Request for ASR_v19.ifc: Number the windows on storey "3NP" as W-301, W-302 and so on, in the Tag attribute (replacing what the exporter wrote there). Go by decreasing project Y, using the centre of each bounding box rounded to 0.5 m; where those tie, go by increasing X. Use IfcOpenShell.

First a look at what the model holds.

```python
import ifcopenshell
import ifcopenshell.util.element
import ifcopenshell.util.placement

model = ifcopenshell.open("ASR_v19.ifc")
print(model.schema)
storey = next(s for s in model.by_type("IfcBuildingStorey") if s.Name == "3NP")
windows = [e for e in ifcopenshell.util.element.get_decomposition(storey) if e.is_a("IfcWindow")]
for e in sorted(windows, key=lambda e: e.id()):
    origin = ifcopenshell.util.placement.get_local_placement(e.ObjectPlacement)[:3, 3]
    print(e.id(), e.Tag, e.Name, origin.round(2) + 0.0, sep=" | ")
```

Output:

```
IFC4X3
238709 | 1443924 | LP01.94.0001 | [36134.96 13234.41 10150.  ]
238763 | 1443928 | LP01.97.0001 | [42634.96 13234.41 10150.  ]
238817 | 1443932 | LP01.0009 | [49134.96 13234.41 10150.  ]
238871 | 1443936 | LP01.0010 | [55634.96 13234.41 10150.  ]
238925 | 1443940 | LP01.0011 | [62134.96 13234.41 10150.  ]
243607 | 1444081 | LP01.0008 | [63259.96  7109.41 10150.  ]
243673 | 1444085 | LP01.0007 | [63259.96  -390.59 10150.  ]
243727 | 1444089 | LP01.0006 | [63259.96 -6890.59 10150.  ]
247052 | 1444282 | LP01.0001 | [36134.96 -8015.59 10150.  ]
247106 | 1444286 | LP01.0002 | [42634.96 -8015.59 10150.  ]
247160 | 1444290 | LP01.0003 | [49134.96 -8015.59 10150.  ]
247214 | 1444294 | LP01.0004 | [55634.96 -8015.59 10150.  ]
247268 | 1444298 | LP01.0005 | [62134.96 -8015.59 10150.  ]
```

```python
import ifcopenshell
import ifcopenshell.geom
import ifcopenshell.util.element
import ifcopenshell.util.shape

model = ifcopenshell.open("ASR_v19.ifc")
settings = ifcopenshell.geom.settings()
settings.set("use-world-coords", True)


def centre(element):
    shape = ifcopenshell.geom.create_shape(settings, element)
    return ifcopenshell.util.shape.get_bbox_centroid(shape.geometry)


storey = next(s for s in model.by_type("IfcBuildingStorey") if s.Name == "3NP")
windows = [e for e in ifcopenshell.util.element.get_decomposition(storey) if e.is_a("IfcWindow")]

# Insertion points can sit at a corner or the storey origin, so sort by the geometry (in metres).
centres = {e: centre(e) for e in windows}
windows.sort(key=lambda e: (-round(centres[e][1] / 0.5), centres[e][0]))

for i, e in enumerate(windows, start=1):
    number = f"W-3{i:02d}"
    e.Tag = number
    print(e.id(), number)

model.write("ASR_v19_updated.ifc")
```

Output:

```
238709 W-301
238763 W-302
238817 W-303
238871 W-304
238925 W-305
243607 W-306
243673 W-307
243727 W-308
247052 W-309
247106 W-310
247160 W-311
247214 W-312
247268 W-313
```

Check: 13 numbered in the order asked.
